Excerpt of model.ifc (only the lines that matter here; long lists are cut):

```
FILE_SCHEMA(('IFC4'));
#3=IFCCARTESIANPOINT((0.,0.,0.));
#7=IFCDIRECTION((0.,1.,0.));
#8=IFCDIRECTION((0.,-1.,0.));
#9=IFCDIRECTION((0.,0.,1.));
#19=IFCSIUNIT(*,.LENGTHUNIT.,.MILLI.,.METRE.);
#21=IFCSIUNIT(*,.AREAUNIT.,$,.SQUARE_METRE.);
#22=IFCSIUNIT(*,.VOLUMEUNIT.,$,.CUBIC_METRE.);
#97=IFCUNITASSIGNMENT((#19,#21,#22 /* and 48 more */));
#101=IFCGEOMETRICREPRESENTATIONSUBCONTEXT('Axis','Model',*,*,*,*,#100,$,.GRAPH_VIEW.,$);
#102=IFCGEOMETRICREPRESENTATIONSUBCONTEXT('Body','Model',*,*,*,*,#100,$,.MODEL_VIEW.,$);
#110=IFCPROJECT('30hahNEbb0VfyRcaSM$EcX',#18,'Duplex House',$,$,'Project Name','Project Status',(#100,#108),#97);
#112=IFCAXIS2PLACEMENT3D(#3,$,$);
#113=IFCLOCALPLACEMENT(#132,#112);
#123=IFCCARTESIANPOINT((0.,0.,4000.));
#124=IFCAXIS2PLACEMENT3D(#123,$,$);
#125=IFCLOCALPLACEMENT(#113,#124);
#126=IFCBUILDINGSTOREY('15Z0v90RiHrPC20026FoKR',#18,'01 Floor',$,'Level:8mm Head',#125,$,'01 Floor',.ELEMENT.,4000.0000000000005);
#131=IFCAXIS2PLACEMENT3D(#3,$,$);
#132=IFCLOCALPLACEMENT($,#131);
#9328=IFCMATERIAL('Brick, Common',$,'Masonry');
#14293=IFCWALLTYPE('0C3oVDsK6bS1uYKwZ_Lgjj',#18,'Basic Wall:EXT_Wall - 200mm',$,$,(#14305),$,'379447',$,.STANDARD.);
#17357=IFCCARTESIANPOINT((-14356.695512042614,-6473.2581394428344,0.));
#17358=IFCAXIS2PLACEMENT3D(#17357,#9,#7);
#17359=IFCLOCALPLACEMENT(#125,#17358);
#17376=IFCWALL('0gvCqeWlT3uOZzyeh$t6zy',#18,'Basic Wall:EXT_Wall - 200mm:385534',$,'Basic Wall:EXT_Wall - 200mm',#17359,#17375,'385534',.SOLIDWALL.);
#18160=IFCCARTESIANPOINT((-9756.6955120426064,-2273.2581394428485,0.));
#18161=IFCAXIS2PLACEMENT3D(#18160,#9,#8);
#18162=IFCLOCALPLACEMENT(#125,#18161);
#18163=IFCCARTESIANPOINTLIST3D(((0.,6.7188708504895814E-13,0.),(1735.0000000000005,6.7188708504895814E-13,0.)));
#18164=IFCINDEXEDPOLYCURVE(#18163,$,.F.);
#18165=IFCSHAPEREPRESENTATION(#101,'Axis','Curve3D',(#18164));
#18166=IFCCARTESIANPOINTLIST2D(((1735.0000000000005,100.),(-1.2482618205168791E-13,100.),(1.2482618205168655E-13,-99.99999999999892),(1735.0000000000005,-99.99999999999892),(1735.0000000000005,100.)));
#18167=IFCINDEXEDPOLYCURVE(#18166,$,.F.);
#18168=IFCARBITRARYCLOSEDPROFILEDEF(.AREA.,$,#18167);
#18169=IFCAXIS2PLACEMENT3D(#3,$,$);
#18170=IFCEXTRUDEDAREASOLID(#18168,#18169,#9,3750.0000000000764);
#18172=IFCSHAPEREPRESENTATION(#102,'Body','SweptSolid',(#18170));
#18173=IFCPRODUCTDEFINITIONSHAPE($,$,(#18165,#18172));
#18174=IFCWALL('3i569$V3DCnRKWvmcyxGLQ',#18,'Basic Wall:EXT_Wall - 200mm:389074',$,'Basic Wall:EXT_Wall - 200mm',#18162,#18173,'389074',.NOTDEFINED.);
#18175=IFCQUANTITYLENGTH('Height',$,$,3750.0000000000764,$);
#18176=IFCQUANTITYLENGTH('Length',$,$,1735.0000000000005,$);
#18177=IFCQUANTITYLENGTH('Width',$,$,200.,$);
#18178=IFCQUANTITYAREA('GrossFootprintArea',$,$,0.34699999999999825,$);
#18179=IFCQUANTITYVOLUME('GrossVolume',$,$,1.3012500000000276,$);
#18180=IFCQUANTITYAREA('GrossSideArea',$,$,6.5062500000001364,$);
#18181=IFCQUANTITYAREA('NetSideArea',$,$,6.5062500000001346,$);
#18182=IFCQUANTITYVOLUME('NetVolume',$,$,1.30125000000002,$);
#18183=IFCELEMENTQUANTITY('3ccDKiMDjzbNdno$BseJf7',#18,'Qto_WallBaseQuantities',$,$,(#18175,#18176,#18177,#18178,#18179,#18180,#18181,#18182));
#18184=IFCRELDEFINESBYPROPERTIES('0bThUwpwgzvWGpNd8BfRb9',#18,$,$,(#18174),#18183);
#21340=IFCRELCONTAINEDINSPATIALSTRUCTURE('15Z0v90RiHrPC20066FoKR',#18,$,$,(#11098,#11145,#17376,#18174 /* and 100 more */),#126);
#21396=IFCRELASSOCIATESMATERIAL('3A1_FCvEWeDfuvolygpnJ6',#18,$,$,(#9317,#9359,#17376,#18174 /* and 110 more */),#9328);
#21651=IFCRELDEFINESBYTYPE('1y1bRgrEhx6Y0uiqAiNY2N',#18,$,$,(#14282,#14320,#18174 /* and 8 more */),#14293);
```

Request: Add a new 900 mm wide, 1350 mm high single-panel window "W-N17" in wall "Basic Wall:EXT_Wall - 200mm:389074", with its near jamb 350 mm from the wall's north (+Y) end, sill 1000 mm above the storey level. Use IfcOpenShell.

```python
import numpy as np
import ifcopenshell
import ifcopenshell.api.feature
import ifcopenshell.api.geometry
import ifcopenshell.api.pset
import ifcopenshell.api.root
import ifcopenshell.api.spatial
import ifcopenshell.geom
import ifcopenshell.util.element
import ifcopenshell.util.placement
import ifcopenshell.util.representation
import ifcopenshell.util.shape
import ifcopenshell.util.unit

model = ifcopenshell.open("model.ifc")
unit_scale = ifcopenshell.util.unit.calculate_unit_scale(model)
area_scale = ifcopenshell.util.unit.calculate_unit_scale(model, "AREAUNIT")
volume_scale = ifcopenshell.util.unit.calculate_unit_scale(model, "VOLUMEUNIT")
settings = ifcopenshell.geom.settings()


def volume(element):
    """Net volume in cubic metres, openings subtracted."""
    shape = ifcopenshell.geom.create_shape(settings, element)
    return ifcopenshell.util.shape.get_volume(shape.geometry)


wall = model.by_id(18174)
storey = ifcopenshell.util.element.get_container(wall, ifc_class="IfcBuildingStorey")
context = ifcopenshell.util.representation.get_context(model, "Model", "Body", "MODEL_VIEW")
before = volume(wall)

width, height, from_end, sill = 0.9, 1.35, 0.35, 1  # metres

# The wall runs along its own X axis, and the end named is its -X end.
wall_shape = ifcopenshell.geom.create_shape(settings, wall)
x, y, z = ifcopenshell.util.shape.get_vertices(wall_shape.geometry).T
start = x.min() + from_end
face, thickness = float(y.min()), float(y.max() - y.min())
wall_matrix = ifcopenshell.util.placement.get_local_placement(wall.ObjectPlacement)
level = ifcopenshell.util.placement.get_local_placement(storey.ObjectPlacement)[2, 3]


def in_wall(x, y):
    """Placement at x, y metres in the wall's axes, at sill height."""
    matrix = wall_matrix.copy()
    matrix[:, 3] = wall_matrix @ np.array([x / unit_scale, y / unit_scale, 0.0, 1.0])
    matrix[2, 3] = level + sill / unit_scale
    return matrix


# Opening: a box that overshoots both wall faces by 50 mm.
opening = ifcopenshell.api.root.create_entity(model, ifc_class="IfcOpeningElement", predefined_type="OPENING")
box = ifcopenshell.api.geometry.add_wall_representation(
    model, context=context, length=width, height=height, thickness=thickness + 0.1
)
ifcopenshell.api.geometry.assign_representation(model, product=opening, representation=box)
ifcopenshell.api.geometry.edit_object_placement(model, product=opening, matrix=in_wall(start, face - 0.05), is_si=False)
ifcopenshell.api.feature.add_feature(model, feature=opening, element=wall)

window = ifcopenshell.api.root.create_entity(model, ifc_class="IfcWindow", name="W-N17", predefined_type="WINDOW")
window.OverallWidth, window.OverallHeight = width / unit_scale, height / unit_scale
window.PartitioningType = "SINGLE_PANEL"
body = ifcopenshell.api.geometry.add_window_representation(
    model,
    context=context,
    overall_width=window.OverallWidth,
    overall_height=window.OverallHeight,
    partition_type="SINGLE_PANEL",
)
ifcopenshell.api.geometry.assign_representation(model, product=window, representation=body)
ifcopenshell.api.spatial.assign_container(model, products=[window], relating_structure=storey)
ifcopenshell.api.feature.add_filling(model, opening=opening, element=window)

# Centre the window in the wall's thickness.
ifcopenshell.api.geometry.edit_object_placement(model, product=window, matrix=in_wall(start, face), is_si=False)
window_shape = ifcopenshell.geom.create_shape(settings, window)
depth = ifcopenshell.util.shape.get_vertices(window_shape.geometry)[:, 1]
offset = face + thickness / 2 - (depth.min() + depth.max()) / 2
ifcopenshell.api.geometry.edit_object_placement(model, product=window, matrix=in_wall(start, offset), is_si=False)

after = volume(wall)

# Update the wall's stored quantities.
qto = model.by_id(ifcopenshell.util.element.get_pset(wall, "Qto_WallBaseQuantities", should_inherit=False)["id"])
ifcopenshell.api.pset.edit_qto(model, qto=qto, properties={
    "NetSideArea": after / thickness / area_scale,
    "NetVolume": after / volume_scale,
})

print(f"wall volume {before:.3f} -> {after:.3f} m3")

model.write("model_updated.ifc")
```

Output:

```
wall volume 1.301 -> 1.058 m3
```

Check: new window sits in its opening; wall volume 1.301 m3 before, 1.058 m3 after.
